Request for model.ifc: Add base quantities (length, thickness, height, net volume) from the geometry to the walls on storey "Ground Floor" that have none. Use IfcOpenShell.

First a look at what the model holds.

```python
import ifcopenshell
import ifcopenshell.util.element
import ifcopenshell.util.unit

model = ifcopenshell.open("model.ifc")
print(model.schema)
for unit_type in ("LENGTHUNIT", "AREAUNIT", "VOLUMEUNIT"):
    print(unit_type, ifcopenshell.util.unit.calculate_unit_scale(model, unit_type))
storey = next(s for s in model.by_type("IfcBuildingStorey") if s.Name == "Ground Floor")
walls = [e for e in ifcopenshell.util.element.get_decomposition(storey) if e.is_a("IfcWall")]
for e in sorted(walls, key=lambda e: e.id()):
    print(e.id(), e.is_a(), e.Name, list(ifcopenshell.util.element.get_psets(e, qtos_only=True)), sep=" | ")
```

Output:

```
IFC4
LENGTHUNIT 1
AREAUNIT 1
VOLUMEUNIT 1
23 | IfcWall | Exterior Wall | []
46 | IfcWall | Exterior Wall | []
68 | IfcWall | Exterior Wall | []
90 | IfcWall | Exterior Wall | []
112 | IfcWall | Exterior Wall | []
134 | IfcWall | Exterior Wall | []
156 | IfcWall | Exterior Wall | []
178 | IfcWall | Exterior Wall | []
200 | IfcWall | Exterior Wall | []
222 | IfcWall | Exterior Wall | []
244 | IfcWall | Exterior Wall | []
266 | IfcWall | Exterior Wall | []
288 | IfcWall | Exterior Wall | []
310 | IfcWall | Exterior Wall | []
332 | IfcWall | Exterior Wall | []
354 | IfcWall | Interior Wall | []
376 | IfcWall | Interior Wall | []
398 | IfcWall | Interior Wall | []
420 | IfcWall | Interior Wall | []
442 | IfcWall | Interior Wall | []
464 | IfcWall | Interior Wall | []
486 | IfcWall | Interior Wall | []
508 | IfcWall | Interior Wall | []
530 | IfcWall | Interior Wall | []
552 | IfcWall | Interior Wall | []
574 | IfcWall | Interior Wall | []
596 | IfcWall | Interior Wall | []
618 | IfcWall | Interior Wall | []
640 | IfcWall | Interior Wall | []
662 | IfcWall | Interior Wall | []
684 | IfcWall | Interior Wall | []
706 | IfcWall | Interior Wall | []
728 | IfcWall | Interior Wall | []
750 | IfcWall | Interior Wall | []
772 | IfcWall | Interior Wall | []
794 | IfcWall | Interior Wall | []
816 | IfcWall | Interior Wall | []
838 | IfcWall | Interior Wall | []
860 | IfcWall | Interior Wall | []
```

```python
import ifcopenshell
import ifcopenshell.api.pset
import ifcopenshell.geom
import ifcopenshell.util.element
import ifcopenshell.util.shape
import ifcopenshell.util.unit

model = ifcopenshell.open("model.ifc")
unit_scale = ifcopenshell.util.unit.calculate_unit_scale(model)
volume_scale = ifcopenshell.util.unit.calculate_unit_scale(model, "VOLUMEUNIT")
settings = ifcopenshell.geom.settings()

storey = next(s for s in model.by_type("IfcBuildingStorey") if s.Name == "Ground Floor")
walls = [e for e in ifcopenshell.util.element.get_decomposition(storey) if e.is_a("IfcWall")]

for e in sorted(walls, key=lambda e: e.id()):
    if ifcopenshell.util.element.get_psets(e, qtos_only=True, should_inherit=False):
        continue
    # Geometry comes back in metres, in the element's own axes.
    shape = ifcopenshell.geom.create_shape(settings, e)
    values = {
        "Length": ifcopenshell.util.shape.get_x(shape.geometry) / unit_scale,
        "Width": ifcopenshell.util.shape.get_y(shape.geometry) / unit_scale,
        "Height": ifcopenshell.util.shape.get_z(shape.geometry) / unit_scale,
        "NetVolume": ifcopenshell.util.shape.get_volume(shape.geometry) / volume_scale,
    }
    qto = ifcopenshell.api.pset.add_qto(model, product=e, name="Qto_WallBaseQuantities")
    ifcopenshell.api.pset.edit_qto(model, qto=qto, properties=values)
    print(e.id(), {k: round(v, 3) for k, v in values.items()})

model.write("model_rev.ifc")
```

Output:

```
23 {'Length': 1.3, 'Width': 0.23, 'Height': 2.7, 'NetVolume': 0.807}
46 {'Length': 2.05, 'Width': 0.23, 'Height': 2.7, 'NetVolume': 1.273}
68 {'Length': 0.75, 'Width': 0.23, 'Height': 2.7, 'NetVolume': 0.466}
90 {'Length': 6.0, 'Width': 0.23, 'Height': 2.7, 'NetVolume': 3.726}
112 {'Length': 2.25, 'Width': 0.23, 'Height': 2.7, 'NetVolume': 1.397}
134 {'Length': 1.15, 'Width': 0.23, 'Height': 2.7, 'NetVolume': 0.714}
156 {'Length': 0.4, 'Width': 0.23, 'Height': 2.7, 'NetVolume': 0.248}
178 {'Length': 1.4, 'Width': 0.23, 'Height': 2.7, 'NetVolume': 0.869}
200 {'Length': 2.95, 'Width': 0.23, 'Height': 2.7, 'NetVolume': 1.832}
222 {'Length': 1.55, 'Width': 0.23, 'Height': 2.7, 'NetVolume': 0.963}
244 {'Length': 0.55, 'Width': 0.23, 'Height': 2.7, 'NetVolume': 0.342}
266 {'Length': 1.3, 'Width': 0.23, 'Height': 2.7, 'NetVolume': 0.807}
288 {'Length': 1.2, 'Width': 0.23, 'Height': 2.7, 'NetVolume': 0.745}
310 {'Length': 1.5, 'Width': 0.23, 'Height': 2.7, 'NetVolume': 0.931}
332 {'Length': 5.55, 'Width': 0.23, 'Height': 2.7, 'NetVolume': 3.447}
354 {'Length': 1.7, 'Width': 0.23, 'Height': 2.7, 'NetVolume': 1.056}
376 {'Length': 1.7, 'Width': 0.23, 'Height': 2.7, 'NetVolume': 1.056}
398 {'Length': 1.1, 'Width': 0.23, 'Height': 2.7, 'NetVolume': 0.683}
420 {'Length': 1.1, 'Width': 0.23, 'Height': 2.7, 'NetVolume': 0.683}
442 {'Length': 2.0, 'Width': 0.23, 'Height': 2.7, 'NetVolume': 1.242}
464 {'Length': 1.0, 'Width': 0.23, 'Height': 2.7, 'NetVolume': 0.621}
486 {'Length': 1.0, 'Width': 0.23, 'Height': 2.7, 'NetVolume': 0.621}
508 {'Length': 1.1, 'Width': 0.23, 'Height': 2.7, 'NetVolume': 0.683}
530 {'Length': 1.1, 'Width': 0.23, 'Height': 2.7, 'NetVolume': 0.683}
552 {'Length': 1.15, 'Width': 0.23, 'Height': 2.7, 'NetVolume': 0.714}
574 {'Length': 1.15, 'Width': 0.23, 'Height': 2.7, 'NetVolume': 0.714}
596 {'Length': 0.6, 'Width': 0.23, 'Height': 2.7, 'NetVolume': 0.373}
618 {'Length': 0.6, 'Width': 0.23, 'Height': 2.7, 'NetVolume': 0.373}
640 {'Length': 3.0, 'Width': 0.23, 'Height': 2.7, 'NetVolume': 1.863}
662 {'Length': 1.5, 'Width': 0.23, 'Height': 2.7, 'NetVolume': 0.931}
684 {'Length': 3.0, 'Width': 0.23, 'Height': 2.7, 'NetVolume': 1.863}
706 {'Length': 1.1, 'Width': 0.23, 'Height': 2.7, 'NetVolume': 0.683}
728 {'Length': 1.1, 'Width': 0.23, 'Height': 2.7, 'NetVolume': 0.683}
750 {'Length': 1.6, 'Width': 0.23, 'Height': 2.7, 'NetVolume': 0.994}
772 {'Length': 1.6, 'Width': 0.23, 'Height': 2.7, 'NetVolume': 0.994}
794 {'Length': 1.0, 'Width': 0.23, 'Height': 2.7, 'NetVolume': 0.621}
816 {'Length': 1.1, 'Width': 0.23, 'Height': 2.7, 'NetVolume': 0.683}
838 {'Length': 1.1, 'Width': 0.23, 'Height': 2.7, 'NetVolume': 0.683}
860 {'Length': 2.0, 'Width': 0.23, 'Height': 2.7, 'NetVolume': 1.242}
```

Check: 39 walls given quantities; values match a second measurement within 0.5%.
